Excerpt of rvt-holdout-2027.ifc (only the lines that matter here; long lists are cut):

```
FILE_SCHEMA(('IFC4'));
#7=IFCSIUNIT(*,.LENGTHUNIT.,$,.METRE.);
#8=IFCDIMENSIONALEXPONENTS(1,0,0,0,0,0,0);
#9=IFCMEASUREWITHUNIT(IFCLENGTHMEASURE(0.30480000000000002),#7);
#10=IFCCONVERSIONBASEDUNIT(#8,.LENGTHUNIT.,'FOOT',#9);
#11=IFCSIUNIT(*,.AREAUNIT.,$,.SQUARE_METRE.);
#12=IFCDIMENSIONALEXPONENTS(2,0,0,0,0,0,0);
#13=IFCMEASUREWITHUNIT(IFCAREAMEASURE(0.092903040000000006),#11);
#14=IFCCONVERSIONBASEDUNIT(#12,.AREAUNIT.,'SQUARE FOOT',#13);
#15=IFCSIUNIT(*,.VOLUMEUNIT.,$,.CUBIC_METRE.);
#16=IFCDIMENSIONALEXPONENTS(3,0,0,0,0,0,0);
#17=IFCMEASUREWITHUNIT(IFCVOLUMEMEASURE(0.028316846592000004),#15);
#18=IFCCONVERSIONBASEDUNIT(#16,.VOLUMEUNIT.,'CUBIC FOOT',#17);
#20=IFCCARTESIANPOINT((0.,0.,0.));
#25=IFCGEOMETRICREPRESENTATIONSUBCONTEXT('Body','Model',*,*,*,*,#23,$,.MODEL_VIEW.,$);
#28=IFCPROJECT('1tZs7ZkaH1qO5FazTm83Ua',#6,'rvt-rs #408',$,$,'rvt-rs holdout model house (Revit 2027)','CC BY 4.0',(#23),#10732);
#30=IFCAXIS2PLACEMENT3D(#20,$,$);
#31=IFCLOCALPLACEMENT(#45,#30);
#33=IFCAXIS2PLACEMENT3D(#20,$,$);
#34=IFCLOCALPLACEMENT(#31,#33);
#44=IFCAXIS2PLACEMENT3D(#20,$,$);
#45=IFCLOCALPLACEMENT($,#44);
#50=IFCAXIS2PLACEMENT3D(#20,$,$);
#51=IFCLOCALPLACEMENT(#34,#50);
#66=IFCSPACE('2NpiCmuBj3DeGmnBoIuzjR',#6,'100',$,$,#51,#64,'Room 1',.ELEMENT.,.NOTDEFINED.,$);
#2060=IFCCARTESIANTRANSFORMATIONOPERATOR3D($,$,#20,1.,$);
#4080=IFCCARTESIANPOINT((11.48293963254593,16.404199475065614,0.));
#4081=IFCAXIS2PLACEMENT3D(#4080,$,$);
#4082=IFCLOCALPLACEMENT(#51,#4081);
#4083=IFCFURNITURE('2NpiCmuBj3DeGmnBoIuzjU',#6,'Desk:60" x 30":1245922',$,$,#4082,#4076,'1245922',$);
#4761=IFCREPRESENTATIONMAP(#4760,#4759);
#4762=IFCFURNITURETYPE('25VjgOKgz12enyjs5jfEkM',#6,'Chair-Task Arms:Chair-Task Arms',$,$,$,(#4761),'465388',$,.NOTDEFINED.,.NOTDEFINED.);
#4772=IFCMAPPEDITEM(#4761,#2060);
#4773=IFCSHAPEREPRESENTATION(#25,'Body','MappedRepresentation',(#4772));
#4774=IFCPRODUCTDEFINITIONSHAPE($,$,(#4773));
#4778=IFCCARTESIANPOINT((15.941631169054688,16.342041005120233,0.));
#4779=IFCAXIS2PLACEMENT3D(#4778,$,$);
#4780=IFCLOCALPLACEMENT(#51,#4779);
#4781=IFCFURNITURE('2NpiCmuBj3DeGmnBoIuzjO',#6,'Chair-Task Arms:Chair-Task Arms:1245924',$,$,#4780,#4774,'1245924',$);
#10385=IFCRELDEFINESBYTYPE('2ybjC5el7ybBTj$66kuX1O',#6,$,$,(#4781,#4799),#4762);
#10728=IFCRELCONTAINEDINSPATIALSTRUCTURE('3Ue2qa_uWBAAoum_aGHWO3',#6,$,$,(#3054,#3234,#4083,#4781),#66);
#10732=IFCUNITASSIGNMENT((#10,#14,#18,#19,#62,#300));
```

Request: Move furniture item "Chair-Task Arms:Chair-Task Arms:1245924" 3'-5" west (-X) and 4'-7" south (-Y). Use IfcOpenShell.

```python
import ifcopenshell
import ifcopenshell.api.geometry
import ifcopenshell.util.placement
import ifcopenshell.util.unit

model = ifcopenshell.open("rvt-holdout-2027.ifc")
unit_scale = ifcopenshell.util.unit.calculate_unit_scale(model)

item = model.by_id(4781)
matrix = ifcopenshell.util.placement.get_local_placement(item.ObjectPlacement)
matrix[0, 3] -= 41 * 0.0254 / unit_scale
matrix[1, 3] -= 55 * 0.0254 / unit_scale
ifcopenshell.api.geometry.edit_object_placement(model, product=item, matrix=matrix, is_si=False)

print(ifcopenshell.util.placement.get_local_placement(item.ObjectPlacement).round(3) + 0.0)

model.write("rvt-holdout-2027_rev.ifc")
```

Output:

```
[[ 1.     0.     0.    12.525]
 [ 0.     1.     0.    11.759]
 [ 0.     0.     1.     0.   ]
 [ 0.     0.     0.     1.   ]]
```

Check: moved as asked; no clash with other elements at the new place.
